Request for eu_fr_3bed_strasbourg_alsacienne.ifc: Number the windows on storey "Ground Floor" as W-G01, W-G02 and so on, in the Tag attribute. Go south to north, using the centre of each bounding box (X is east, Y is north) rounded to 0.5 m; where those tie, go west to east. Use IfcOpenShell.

First a look at what the model holds.

```python
import ifcopenshell
import ifcopenshell.util.element
import ifcopenshell.util.placement

model = ifcopenshell.open("eu_fr_3bed_strasbourg_alsacienne.ifc")
print(model.schema)
storey = next(s for s in model.by_type("IfcBuildingStorey") if s.Name == "Ground Floor")
windows = [e for e in ifcopenshell.util.element.get_decomposition(storey) if e.is_a("IfcWindow")]
for e in sorted(windows, key=lambda e: e.id()):
    origin = ifcopenshell.util.placement.get_local_placement(e.ObjectPlacement)[:3, 3]
    print(e.id(), e.Tag, e.Name, origin.round(2) + 0.0, sep=" | ")
```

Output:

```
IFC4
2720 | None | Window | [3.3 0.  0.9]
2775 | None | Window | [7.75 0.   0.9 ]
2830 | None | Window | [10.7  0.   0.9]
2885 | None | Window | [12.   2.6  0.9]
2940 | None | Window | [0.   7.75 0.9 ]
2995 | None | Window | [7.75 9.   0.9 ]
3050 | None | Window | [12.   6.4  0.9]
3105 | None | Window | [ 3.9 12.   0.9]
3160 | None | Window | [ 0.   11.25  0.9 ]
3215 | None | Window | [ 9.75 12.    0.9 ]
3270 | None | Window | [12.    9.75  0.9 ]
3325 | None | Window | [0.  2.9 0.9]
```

```python
import ifcopenshell
import ifcopenshell.geom
import ifcopenshell.util.element
import ifcopenshell.util.shape

model = ifcopenshell.open("eu_fr_3bed_strasbourg_alsacienne.ifc")
settings = ifcopenshell.geom.settings()
settings.set("use-world-coords", True)


def centre(element):
    shape = ifcopenshell.geom.create_shape(settings, element)
    return ifcopenshell.util.shape.get_bbox_centroid(shape.geometry)


storey = next(s for s in model.by_type("IfcBuildingStorey") if s.Name == "Ground Floor")
windows = [e for e in ifcopenshell.util.element.get_decomposition(storey) if e.is_a("IfcWindow")]

# Insertion points can sit at a corner or the storey origin, so sort by the geometry (in metres).
centres = {e: centre(e) for e in windows}
windows.sort(key=lambda e: (round(centres[e][1] / 0.5), centres[e][0]))

for i, e in enumerate(windows, start=1):
    number = f"W-G{i:02d}"
    e.Tag = number
    print(e.id(), number)

model.write("eu_fr_3bed_strasbourg_alsacienne_rev.ifc")
```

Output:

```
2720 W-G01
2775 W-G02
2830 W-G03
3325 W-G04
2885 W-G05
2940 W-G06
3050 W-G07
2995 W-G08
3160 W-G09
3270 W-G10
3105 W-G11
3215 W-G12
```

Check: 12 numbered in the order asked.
